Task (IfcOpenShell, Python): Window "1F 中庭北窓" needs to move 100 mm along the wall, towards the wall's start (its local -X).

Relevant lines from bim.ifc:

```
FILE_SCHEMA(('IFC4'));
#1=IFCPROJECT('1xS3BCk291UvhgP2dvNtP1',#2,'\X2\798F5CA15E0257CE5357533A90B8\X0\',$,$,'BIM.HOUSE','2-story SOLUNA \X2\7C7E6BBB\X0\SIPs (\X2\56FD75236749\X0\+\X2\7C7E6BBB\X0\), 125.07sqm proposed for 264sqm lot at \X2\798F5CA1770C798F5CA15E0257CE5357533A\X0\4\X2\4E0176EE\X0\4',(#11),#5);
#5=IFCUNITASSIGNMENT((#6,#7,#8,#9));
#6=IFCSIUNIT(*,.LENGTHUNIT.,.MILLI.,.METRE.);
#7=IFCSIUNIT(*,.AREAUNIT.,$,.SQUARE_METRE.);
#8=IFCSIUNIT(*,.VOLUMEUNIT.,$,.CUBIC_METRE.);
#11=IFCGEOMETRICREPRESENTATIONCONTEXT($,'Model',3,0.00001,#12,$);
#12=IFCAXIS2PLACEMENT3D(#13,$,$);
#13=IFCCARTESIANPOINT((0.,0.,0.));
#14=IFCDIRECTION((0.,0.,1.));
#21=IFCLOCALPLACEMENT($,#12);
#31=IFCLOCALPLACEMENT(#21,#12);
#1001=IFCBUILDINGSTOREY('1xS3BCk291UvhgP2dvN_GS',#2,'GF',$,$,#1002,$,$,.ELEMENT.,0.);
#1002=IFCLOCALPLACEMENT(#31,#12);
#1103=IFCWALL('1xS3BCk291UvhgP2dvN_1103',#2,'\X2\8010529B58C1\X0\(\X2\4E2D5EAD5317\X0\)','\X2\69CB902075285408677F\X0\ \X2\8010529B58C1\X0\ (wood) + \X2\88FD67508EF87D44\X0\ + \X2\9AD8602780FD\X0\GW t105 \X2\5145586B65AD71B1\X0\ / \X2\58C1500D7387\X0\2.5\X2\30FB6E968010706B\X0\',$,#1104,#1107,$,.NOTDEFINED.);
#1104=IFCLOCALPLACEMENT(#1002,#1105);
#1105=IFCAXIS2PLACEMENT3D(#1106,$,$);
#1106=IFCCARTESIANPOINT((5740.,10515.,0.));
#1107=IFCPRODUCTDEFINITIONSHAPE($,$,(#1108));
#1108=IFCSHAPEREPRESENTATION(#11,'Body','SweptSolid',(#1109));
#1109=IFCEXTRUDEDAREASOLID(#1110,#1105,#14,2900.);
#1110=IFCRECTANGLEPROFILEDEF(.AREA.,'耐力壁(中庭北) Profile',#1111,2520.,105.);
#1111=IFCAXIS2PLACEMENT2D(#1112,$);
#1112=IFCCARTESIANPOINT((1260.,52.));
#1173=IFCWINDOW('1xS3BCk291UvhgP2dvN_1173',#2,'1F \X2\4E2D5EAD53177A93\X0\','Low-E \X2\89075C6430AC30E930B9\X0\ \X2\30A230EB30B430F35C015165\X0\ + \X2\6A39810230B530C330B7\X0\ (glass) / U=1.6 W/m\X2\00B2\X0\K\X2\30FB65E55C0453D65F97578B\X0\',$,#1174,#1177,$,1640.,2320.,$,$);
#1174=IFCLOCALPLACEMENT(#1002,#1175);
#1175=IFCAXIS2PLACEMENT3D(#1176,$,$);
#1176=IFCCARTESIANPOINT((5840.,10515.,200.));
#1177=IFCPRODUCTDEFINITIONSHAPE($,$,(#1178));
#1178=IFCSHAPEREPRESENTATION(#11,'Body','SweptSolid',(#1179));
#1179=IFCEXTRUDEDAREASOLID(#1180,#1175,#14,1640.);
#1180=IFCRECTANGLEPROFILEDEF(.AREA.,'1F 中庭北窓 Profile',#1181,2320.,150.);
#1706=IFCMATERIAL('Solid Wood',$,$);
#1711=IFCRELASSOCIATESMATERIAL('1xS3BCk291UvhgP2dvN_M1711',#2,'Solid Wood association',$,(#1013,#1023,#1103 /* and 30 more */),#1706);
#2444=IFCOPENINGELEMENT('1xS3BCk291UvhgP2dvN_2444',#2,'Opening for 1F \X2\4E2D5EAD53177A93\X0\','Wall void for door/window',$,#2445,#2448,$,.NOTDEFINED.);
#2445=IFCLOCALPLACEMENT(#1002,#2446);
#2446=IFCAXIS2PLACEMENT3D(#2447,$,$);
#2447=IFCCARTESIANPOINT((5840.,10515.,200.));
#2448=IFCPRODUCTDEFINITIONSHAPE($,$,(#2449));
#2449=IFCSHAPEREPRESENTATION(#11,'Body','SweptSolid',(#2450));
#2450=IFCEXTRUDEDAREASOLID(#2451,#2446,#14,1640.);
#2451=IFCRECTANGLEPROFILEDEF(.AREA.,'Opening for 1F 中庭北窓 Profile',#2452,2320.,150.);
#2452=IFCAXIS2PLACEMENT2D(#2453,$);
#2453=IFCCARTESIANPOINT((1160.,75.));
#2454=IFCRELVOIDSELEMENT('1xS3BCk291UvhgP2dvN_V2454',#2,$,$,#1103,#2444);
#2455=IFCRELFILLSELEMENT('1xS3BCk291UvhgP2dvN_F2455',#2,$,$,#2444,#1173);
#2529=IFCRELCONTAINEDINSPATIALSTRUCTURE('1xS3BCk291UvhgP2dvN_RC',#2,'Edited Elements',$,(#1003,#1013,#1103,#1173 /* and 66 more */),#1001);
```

```python
import ifcopenshell
import ifcopenshell.api.geometry
import ifcopenshell.util.placement
import ifcopenshell.util.unit

model = ifcopenshell.open("bim.ifc")
unit_scale = ifcopenshell.util.unit.calculate_unit_scale(model)

window = model.by_guid("1xS3BCk291UvhgP2dvN_1173")
opening = window.FillsVoids[0].RelatingOpeningElement
wall = opening.VoidsElements[0].RelatingBuildingElement

wall_matrix = ifcopenshell.util.placement.get_local_placement(wall.ObjectPlacement)
shift = wall_matrix[:3, 0] * -0.1 / unit_scale
before = ifcopenshell.util.placement.get_local_placement(window.ObjectPlacement)[:3, 3].copy()

# The window is not placed relative to its opening, so move both.
for product in (opening, window):
    matrix = ifcopenshell.util.placement.get_local_placement(product.ObjectPlacement)
    matrix[:3, 3] += shift
    ifcopenshell.api.geometry.edit_object_placement(model, product=product, matrix=matrix, is_si=False)

after = ifcopenshell.util.placement.get_local_placement(window.ObjectPlacement)[:3, 3]
print("window moved by", (after - before).round(3) + 0.0)

model.write("bim_rev.ifc")
```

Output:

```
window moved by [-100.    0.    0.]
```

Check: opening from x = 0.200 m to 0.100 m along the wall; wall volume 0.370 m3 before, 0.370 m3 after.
